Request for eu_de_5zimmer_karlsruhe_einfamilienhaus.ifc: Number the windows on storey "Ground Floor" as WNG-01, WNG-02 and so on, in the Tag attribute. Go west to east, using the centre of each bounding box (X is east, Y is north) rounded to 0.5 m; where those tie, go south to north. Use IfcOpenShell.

First a look at what the model holds.

```python
import ifcopenshell
import ifcopenshell.util.element
import ifcopenshell.util.placement

model = ifcopenshell.open("eu_de_5zimmer_karlsruhe_einfamilienhaus.ifc")
print(model.schema)
storey = next(s for s in model.by_type("IfcBuildingStorey") if s.Name == "Ground Floor")
windows = [e for e in ifcopenshell.util.element.get_decomposition(storey) if e.is_a("IfcWindow")]
for e in sorted(windows, key=lambda e: e.id()):
    origin = ifcopenshell.util.placement.get_local_placement(e.ObjectPlacement)[:3, 3]
    print(e.id(), e.Tag, e.Name, origin.round(2) + 0.0, sep=" | ")
```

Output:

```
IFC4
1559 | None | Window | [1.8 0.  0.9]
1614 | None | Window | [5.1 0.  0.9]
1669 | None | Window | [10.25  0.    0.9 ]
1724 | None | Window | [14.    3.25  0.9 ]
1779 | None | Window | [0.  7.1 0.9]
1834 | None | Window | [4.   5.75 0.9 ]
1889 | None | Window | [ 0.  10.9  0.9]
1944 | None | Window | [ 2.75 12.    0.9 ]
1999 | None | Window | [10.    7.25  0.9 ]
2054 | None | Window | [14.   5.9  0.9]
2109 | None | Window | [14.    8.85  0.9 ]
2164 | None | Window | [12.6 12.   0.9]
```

```python
import ifcopenshell
import ifcopenshell.geom
import ifcopenshell.util.element
import ifcopenshell.util.shape

model = ifcopenshell.open("eu_de_5zimmer_karlsruhe_einfamilienhaus.ifc")
settings = ifcopenshell.geom.settings()
settings.set("use-world-coords", True)


def centre(element):
    shape = ifcopenshell.geom.create_shape(settings, element)
    return ifcopenshell.util.shape.get_bbox_centroid(shape.geometry)


storey = next(s for s in model.by_type("IfcBuildingStorey") if s.Name == "Ground Floor")
windows = [e for e in ifcopenshell.util.element.get_decomposition(storey) if e.is_a("IfcWindow")]

# Insertion points can sit at a corner or the storey origin, so sort by the geometry (in metres).
centres = {e: centre(e) for e in windows}
windows.sort(key=lambda e: (round(centres[e][0] / 0.5), centres[e][1]))

for i, e in enumerate(windows, start=1):
    number = f"WNG-{i:02d}"
    e.Tag = number
    print(e.id(), number)

model.write("eu_de_5zimmer_karlsruhe_einfamilienhaus_rev.ifc")
```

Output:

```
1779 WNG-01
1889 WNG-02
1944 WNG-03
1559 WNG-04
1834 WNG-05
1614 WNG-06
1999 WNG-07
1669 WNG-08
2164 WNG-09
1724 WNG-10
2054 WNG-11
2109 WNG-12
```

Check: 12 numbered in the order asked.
